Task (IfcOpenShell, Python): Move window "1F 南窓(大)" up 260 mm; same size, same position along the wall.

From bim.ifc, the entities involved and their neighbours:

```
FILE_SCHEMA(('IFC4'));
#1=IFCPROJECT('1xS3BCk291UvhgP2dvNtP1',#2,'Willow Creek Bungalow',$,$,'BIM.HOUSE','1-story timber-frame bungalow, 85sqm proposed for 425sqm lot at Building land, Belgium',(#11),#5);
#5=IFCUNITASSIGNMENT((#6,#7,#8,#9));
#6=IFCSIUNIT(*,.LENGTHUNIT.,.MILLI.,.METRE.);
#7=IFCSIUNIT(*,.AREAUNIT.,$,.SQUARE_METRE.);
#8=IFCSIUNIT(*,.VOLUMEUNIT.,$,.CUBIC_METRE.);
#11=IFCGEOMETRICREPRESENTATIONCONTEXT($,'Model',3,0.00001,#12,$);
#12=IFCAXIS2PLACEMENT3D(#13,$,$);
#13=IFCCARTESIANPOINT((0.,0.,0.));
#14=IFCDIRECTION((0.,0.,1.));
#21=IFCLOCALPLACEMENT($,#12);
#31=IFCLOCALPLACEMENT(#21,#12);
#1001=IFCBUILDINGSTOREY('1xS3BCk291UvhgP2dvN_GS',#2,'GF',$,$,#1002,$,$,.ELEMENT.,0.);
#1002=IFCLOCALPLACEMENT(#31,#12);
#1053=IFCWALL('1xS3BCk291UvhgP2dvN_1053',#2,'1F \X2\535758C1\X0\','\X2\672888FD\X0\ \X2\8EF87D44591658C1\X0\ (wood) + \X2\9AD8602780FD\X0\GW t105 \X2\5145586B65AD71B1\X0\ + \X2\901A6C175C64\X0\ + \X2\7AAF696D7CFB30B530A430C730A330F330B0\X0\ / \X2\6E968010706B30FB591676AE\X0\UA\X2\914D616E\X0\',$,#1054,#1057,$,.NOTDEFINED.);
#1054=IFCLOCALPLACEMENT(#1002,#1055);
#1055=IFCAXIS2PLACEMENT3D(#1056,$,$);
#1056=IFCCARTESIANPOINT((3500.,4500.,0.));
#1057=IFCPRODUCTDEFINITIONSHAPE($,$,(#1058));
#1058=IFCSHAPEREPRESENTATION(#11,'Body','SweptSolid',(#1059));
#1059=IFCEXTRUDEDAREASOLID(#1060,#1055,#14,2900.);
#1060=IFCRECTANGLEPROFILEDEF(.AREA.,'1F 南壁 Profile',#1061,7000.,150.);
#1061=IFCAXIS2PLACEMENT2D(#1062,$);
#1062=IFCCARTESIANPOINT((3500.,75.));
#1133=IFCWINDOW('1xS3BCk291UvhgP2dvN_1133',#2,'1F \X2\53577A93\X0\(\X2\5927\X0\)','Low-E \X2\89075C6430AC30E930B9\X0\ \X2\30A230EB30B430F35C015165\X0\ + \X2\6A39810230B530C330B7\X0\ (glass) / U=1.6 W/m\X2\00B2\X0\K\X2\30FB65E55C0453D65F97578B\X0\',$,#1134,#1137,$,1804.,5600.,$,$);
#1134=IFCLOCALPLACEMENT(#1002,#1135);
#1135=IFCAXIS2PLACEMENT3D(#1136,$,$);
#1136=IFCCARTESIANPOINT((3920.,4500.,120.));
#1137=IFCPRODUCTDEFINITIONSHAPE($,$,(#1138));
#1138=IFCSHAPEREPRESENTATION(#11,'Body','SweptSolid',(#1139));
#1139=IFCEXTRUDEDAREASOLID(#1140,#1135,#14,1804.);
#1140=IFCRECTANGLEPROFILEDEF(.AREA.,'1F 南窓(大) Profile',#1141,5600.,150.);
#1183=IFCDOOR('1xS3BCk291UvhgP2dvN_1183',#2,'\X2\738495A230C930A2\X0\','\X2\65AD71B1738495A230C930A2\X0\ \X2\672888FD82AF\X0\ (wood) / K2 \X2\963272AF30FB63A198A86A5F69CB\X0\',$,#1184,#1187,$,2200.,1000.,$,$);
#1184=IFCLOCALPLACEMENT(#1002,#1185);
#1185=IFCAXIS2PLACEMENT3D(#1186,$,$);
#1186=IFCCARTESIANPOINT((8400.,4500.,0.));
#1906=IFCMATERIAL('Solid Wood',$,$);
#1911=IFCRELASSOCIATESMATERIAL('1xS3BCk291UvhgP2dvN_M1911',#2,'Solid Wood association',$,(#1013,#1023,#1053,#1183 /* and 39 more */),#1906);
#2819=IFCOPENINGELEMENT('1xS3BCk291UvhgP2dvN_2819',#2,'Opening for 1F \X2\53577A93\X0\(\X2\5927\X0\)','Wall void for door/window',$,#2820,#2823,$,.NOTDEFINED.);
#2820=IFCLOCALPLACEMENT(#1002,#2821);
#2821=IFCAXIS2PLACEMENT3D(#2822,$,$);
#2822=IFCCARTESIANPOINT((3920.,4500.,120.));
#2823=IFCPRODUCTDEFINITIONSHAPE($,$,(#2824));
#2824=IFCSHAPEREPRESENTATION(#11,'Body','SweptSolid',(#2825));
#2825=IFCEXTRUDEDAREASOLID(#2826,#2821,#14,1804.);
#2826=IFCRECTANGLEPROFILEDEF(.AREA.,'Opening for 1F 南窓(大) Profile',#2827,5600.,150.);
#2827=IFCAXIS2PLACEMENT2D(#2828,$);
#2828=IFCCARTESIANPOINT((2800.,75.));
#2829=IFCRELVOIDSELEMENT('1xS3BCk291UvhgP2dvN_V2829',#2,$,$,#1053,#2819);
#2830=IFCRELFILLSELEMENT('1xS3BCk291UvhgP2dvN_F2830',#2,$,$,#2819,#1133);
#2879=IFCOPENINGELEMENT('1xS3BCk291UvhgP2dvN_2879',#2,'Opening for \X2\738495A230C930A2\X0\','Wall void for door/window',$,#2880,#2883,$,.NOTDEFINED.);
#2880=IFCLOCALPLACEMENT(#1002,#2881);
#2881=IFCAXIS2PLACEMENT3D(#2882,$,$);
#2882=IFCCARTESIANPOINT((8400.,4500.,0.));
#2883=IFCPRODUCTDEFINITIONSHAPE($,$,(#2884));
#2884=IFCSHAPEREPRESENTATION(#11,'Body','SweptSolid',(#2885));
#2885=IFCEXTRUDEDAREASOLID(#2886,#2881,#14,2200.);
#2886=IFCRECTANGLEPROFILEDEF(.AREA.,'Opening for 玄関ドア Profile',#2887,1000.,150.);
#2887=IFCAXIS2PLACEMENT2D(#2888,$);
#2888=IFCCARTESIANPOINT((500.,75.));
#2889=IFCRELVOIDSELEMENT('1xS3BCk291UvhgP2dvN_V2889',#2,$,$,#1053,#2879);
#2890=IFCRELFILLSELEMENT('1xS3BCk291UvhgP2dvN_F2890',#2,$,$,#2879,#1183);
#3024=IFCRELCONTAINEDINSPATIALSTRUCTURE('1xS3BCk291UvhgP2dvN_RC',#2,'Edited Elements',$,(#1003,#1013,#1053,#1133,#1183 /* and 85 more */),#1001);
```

```python
import numpy as np
import ifcopenshell
import ifcopenshell.api.geometry
import ifcopenshell.util.placement
import ifcopenshell.util.unit

model = ifcopenshell.open("bim.ifc")
unit_scale = ifcopenshell.util.unit.calculate_unit_scale(model)

window = model.by_id(1133)
opening = window.FillsVoids[0].RelatingOpeningElement
dz = 260.0

shift = np.array([0.0, 0.0, dz])
# The window is not placed relative to its opening, so move both.
for product in (opening, window):
    matrix = ifcopenshell.util.placement.get_local_placement(product.ObjectPlacement)
    matrix[:3, 3] += shift
    ifcopenshell.api.geometry.edit_object_placement(model, product=product, matrix=matrix, is_si=False)

print(f"moved by {dz * unit_scale:+.3f} m")

model.write("bim_v2.ifc")
```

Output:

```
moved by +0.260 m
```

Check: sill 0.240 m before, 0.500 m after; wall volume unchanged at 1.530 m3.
